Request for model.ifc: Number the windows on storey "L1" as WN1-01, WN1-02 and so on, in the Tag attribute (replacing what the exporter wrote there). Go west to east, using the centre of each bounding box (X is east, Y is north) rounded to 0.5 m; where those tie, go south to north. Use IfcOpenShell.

First a look at what the model holds.

```python
import ifcopenshell
import ifcopenshell.util.element
import ifcopenshell.util.placement

model = ifcopenshell.open("model.ifc")
print(model.schema)
storey = next(s for s in model.by_type("IfcBuildingStorey") if s.Name == "L1")
windows = [e for e in ifcopenshell.util.element.get_decomposition(storey) if e.is_a("IfcWindow")]
for e in sorted(windows, key=lambda e: e.id()):
    origin = ifcopenshell.util.placement.get_local_placement(e.ObjectPlacement)[:3, 3]
    print(e.id(), e.Tag, e.Name, origin.round(2) + 0.0, sep=" | ")
```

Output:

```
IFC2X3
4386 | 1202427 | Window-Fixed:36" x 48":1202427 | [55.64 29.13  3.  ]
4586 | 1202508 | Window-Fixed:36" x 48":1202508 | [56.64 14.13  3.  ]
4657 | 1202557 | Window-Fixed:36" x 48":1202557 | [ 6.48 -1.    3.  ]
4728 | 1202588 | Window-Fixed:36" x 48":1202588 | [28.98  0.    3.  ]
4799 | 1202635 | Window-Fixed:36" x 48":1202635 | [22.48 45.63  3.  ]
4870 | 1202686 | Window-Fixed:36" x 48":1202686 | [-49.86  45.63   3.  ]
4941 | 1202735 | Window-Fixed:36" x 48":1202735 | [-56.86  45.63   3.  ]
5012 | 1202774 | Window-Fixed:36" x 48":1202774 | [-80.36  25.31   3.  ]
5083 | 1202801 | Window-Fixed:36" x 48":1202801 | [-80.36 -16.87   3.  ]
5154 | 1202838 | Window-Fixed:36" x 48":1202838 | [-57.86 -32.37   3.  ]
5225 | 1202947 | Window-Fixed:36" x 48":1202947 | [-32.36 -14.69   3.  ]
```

```python
import ifcopenshell
import ifcopenshell.geom
import ifcopenshell.util.element
import ifcopenshell.util.shape

model = ifcopenshell.open("model.ifc")
settings = ifcopenshell.geom.settings()
settings.set("use-world-coords", True)


def centre(element):
    shape = ifcopenshell.geom.create_shape(settings, element)
    return ifcopenshell.util.shape.get_bbox_centroid(shape.geometry)


storey = next(s for s in model.by_type("IfcBuildingStorey") if s.Name == "L1")
windows = [e for e in ifcopenshell.util.element.get_decomposition(storey) if e.is_a("IfcWindow")]

# Insertion points can sit at a corner or the storey origin, so sort by the geometry (in metres).
centres = {e: centre(e) for e in windows}
windows.sort(key=lambda e: (round(centres[e][0] / 0.5), centres[e][1]))

for i, e in enumerate(windows, start=1):
    number = f"WN1-{i:02d}"
    e.Tag = number
    print(e.id(), number)

model.write("model_edited.ifc")
```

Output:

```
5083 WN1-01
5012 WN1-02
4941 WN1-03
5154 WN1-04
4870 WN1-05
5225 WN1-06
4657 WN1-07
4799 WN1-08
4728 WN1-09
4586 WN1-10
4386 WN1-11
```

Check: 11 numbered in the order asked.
